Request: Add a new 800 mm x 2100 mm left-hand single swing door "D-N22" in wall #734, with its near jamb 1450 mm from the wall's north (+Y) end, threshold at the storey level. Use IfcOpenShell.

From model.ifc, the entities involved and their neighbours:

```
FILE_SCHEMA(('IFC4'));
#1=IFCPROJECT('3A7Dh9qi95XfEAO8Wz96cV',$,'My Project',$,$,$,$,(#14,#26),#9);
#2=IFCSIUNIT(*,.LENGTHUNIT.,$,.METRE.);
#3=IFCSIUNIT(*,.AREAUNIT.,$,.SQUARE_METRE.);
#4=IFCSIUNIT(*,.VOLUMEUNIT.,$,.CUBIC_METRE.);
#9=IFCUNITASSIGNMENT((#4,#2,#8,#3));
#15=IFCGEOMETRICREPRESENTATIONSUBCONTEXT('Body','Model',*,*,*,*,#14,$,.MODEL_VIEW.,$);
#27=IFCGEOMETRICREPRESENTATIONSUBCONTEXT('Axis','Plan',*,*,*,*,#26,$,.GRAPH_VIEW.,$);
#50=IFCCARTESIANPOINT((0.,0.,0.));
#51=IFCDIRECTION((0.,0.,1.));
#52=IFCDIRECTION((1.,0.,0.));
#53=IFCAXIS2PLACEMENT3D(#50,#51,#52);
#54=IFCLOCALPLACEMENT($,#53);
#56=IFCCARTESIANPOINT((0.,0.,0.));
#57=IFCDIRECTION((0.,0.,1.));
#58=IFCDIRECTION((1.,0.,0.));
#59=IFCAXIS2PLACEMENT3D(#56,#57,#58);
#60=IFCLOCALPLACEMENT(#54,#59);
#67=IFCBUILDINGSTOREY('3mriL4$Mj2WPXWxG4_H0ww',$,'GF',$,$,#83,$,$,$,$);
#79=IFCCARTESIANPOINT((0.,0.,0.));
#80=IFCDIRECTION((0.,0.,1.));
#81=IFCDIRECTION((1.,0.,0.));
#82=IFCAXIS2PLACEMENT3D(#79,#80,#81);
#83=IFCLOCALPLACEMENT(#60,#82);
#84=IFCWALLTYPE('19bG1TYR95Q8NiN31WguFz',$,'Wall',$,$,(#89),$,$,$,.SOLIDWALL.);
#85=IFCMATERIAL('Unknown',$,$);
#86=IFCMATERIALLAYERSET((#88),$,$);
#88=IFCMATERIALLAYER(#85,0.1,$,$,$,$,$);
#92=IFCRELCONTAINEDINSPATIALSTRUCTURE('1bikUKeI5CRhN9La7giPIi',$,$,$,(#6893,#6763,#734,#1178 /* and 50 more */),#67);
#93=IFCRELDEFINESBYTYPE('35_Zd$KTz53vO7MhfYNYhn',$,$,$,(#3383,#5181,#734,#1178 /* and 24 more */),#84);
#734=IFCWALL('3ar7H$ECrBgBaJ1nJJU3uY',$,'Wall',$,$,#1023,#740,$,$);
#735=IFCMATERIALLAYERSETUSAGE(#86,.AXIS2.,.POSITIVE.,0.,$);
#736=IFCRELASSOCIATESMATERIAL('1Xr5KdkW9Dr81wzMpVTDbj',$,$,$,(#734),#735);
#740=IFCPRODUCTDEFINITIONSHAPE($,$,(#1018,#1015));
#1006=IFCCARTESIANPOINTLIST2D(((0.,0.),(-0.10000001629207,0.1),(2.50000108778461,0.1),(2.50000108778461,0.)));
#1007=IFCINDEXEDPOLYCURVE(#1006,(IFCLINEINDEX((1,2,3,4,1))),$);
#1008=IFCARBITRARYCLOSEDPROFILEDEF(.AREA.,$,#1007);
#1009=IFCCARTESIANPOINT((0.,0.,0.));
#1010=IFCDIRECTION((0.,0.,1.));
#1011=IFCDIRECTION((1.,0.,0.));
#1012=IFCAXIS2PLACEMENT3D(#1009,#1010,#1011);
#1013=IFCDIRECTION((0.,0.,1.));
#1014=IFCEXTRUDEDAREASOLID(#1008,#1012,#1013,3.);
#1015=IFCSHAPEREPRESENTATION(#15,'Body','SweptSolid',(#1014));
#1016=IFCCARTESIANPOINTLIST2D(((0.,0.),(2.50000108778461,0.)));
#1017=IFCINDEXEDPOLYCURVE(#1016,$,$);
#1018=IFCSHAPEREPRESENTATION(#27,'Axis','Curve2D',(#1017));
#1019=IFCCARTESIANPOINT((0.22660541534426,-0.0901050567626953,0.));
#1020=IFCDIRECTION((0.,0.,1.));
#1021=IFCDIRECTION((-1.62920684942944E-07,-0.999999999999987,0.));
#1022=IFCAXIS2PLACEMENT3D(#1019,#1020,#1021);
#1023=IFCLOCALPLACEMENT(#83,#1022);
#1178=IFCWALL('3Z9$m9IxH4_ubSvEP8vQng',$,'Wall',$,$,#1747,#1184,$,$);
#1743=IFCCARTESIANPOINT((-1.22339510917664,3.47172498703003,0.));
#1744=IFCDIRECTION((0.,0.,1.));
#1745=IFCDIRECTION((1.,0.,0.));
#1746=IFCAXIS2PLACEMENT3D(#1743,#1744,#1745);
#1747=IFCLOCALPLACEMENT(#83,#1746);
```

```python
import numpy as np
import ifcopenshell
import ifcopenshell.api.feature
import ifcopenshell.api.geometry
import ifcopenshell.api.root
import ifcopenshell.api.spatial
import ifcopenshell.geom
import ifcopenshell.util.element
import ifcopenshell.util.placement
import ifcopenshell.util.representation
import ifcopenshell.util.shape
import ifcopenshell.util.unit

model = ifcopenshell.open("model.ifc")
unit_scale = ifcopenshell.util.unit.calculate_unit_scale(model)
settings = ifcopenshell.geom.settings()


def volume(element):
    """Net volume in cubic metres, openings subtracted."""
    shape = ifcopenshell.geom.create_shape(settings, element)
    return ifcopenshell.util.shape.get_volume(shape.geometry)


wall = model.by_id(734)
storey = ifcopenshell.util.element.get_container(wall, ifc_class="IfcBuildingStorey")
context = ifcopenshell.util.representation.get_context(model, "Model", "Body", "MODEL_VIEW")
before = volume(wall)

width, height, from_end, sill = 0.8, 2.1, 1.45, 0.0  # metres

# The wall runs along its own X axis, and the end named is its -X end.
wall_shape = ifcopenshell.geom.create_shape(settings, wall)
x, y, z = ifcopenshell.util.shape.get_vertices(wall_shape.geometry).T
start = x.min() + from_end
face, thickness = float(y.min()), float(y.max() - y.min())
wall_matrix = ifcopenshell.util.placement.get_local_placement(wall.ObjectPlacement)
level = ifcopenshell.util.placement.get_local_placement(storey.ObjectPlacement)[2, 3]


def in_wall(x, y):
    """Placement at x, y metres in the wall's axes, at sill height."""
    matrix = wall_matrix.copy()
    matrix[:, 3] = wall_matrix @ np.array([x / unit_scale, y / unit_scale, 0.0, 1.0])
    matrix[2, 3] = level + sill / unit_scale
    return matrix


# Opening: a box that overshoots both wall faces by 50 mm.
opening = ifcopenshell.api.root.create_entity(model, ifc_class="IfcOpeningElement", predefined_type="OPENING")
box = ifcopenshell.api.geometry.add_wall_representation(
    model, context=context, length=width, height=height, thickness=thickness + 0.1
)
ifcopenshell.api.geometry.assign_representation(model, product=opening, representation=box)
ifcopenshell.api.geometry.edit_object_placement(model, product=opening, matrix=in_wall(start, face - 0.05), is_si=False)
ifcopenshell.api.feature.add_feature(model, feature=opening, element=wall)

door = ifcopenshell.api.root.create_entity(model, ifc_class="IfcDoor", name="D-N22", predefined_type="DOOR")
door.OverallWidth, door.OverallHeight = width / unit_scale, height / unit_scale
door.OperationType = "SINGLE_SWING_LEFT"
body = ifcopenshell.api.geometry.add_door_representation(
    model,
    context=context,
    overall_width=door.OverallWidth,
    overall_height=door.OverallHeight,
    operation_type="SINGLE_SWING_LEFT",
    lining_properties={"LiningDepth": thickness / unit_scale, "ThresholdDepth": thickness / unit_scale},
)
ifcopenshell.api.geometry.assign_representation(model, product=door, representation=body)
ifcopenshell.api.spatial.assign_container(model, products=[door], relating_structure=storey)
ifcopenshell.api.feature.add_filling(model, opening=opening, element=door)

# The lining spans the wall, so the door starts at the wall face.
ifcopenshell.api.geometry.edit_object_placement(model, product=door, matrix=in_wall(start, face), is_si=False)

after = volume(wall)

print(f"wall volume {before:.3f} -> {after:.3f} m3")

model.write("model_rev.ifc")
```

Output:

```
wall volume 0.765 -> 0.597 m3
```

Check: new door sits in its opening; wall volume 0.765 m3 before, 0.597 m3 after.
